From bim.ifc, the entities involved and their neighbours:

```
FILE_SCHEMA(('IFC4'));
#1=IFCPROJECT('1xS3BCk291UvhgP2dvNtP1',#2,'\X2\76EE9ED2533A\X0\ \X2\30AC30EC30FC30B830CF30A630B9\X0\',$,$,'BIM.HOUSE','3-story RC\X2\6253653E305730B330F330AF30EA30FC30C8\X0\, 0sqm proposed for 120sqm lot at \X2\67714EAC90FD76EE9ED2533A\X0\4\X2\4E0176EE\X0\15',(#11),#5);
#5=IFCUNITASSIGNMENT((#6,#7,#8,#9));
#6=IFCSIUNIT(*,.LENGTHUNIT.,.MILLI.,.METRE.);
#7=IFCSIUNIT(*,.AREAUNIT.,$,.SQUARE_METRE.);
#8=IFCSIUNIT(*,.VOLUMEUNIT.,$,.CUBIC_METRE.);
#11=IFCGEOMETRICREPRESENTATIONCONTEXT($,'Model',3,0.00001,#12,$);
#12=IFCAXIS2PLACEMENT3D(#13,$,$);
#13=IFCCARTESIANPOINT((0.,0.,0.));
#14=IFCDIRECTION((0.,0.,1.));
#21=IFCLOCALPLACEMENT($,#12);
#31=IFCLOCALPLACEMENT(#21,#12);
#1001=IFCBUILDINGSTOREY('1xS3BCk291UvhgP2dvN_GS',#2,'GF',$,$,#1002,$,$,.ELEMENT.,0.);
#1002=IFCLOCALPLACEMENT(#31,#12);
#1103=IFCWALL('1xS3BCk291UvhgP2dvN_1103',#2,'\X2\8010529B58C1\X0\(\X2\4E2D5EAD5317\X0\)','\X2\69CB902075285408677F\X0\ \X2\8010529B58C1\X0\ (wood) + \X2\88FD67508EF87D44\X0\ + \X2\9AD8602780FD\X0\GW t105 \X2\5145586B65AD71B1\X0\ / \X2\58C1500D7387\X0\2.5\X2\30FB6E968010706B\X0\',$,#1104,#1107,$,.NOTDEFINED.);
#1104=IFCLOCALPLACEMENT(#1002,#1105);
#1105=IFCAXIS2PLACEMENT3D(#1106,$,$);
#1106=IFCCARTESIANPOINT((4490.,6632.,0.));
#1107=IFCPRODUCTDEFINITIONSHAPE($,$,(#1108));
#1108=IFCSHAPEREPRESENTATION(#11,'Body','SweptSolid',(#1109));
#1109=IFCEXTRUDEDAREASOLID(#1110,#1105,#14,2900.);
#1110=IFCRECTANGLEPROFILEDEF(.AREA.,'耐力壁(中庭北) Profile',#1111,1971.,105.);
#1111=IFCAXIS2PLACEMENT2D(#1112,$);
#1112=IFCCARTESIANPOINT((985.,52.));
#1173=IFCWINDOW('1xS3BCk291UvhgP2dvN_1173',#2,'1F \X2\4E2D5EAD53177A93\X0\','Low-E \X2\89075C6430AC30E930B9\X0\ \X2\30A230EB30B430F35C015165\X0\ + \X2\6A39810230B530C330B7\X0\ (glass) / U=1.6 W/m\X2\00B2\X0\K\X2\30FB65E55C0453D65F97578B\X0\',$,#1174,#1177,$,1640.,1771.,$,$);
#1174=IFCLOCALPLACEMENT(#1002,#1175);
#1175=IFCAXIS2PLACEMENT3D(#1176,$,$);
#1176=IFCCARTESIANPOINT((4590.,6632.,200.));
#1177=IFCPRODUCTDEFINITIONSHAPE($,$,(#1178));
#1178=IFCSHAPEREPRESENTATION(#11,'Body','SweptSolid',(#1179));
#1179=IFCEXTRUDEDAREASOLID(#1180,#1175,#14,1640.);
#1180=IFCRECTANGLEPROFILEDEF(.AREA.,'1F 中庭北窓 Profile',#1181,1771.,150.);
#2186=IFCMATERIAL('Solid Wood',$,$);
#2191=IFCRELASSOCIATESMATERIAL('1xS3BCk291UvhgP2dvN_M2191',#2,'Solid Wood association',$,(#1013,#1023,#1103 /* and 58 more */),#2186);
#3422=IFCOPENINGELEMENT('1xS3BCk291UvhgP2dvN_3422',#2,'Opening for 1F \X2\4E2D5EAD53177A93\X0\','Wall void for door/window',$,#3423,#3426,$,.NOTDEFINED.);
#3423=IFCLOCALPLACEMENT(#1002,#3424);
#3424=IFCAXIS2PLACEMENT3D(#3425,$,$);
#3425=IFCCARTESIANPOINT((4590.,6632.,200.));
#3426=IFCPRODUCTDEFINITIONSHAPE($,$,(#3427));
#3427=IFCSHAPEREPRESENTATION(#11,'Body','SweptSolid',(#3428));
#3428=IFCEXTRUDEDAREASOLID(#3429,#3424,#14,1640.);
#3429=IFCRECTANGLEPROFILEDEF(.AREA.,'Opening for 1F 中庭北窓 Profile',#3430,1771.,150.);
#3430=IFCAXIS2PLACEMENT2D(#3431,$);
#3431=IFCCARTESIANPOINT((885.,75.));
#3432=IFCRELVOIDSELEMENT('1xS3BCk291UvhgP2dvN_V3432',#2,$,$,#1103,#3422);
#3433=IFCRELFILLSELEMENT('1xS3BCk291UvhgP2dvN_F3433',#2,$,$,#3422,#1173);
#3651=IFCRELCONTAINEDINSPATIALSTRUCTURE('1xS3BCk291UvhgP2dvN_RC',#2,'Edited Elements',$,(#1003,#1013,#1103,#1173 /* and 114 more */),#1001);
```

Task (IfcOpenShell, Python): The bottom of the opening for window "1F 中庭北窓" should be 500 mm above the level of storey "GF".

```python
import numpy as np
import ifcopenshell
import ifcopenshell.api.geometry
import ifcopenshell.geom
import ifcopenshell.util.element
import ifcopenshell.util.placement
import ifcopenshell.util.shape
import ifcopenshell.util.unit

model = ifcopenshell.open("bim.ifc")
unit_scale = ifcopenshell.util.unit.calculate_unit_scale(model)

window = model.by_guid("1xS3BCk291UvhgP2dvN_1173")
opening = window.FillsVoids[0].RelatingOpeningElement
storey = ifcopenshell.util.element.get_container(window, ifc_class="IfcBuildingStorey")
level = ifcopenshell.util.placement.get_local_placement(storey.ObjectPlacement)[2, 3]

# The opening's origin need not be at the sill, so measure its lowest point.
shape = ifcopenshell.geom.create_shape(ifcopenshell.geom.settings(), opening)
bottom = ifcopenshell.util.shape.get_shape_bottom_elevation(shape, shape.geometry) / unit_scale
dz = level + 0.5 / unit_scale - bottom

shift = np.array([0.0, 0.0, dz])
# The window is not placed relative to its opening, so move both.
for product in (opening, window):
    matrix = ifcopenshell.util.placement.get_local_placement(product.ObjectPlacement)
    matrix[:3, 3] += shift
    ifcopenshell.api.geometry.edit_object_placement(model, product=product, matrix=matrix, is_si=False)

print(f"moved by {dz * unit_scale:+.3f} m")

model.write("bim_updated.ifc")
```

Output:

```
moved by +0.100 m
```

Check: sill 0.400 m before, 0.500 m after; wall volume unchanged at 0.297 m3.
